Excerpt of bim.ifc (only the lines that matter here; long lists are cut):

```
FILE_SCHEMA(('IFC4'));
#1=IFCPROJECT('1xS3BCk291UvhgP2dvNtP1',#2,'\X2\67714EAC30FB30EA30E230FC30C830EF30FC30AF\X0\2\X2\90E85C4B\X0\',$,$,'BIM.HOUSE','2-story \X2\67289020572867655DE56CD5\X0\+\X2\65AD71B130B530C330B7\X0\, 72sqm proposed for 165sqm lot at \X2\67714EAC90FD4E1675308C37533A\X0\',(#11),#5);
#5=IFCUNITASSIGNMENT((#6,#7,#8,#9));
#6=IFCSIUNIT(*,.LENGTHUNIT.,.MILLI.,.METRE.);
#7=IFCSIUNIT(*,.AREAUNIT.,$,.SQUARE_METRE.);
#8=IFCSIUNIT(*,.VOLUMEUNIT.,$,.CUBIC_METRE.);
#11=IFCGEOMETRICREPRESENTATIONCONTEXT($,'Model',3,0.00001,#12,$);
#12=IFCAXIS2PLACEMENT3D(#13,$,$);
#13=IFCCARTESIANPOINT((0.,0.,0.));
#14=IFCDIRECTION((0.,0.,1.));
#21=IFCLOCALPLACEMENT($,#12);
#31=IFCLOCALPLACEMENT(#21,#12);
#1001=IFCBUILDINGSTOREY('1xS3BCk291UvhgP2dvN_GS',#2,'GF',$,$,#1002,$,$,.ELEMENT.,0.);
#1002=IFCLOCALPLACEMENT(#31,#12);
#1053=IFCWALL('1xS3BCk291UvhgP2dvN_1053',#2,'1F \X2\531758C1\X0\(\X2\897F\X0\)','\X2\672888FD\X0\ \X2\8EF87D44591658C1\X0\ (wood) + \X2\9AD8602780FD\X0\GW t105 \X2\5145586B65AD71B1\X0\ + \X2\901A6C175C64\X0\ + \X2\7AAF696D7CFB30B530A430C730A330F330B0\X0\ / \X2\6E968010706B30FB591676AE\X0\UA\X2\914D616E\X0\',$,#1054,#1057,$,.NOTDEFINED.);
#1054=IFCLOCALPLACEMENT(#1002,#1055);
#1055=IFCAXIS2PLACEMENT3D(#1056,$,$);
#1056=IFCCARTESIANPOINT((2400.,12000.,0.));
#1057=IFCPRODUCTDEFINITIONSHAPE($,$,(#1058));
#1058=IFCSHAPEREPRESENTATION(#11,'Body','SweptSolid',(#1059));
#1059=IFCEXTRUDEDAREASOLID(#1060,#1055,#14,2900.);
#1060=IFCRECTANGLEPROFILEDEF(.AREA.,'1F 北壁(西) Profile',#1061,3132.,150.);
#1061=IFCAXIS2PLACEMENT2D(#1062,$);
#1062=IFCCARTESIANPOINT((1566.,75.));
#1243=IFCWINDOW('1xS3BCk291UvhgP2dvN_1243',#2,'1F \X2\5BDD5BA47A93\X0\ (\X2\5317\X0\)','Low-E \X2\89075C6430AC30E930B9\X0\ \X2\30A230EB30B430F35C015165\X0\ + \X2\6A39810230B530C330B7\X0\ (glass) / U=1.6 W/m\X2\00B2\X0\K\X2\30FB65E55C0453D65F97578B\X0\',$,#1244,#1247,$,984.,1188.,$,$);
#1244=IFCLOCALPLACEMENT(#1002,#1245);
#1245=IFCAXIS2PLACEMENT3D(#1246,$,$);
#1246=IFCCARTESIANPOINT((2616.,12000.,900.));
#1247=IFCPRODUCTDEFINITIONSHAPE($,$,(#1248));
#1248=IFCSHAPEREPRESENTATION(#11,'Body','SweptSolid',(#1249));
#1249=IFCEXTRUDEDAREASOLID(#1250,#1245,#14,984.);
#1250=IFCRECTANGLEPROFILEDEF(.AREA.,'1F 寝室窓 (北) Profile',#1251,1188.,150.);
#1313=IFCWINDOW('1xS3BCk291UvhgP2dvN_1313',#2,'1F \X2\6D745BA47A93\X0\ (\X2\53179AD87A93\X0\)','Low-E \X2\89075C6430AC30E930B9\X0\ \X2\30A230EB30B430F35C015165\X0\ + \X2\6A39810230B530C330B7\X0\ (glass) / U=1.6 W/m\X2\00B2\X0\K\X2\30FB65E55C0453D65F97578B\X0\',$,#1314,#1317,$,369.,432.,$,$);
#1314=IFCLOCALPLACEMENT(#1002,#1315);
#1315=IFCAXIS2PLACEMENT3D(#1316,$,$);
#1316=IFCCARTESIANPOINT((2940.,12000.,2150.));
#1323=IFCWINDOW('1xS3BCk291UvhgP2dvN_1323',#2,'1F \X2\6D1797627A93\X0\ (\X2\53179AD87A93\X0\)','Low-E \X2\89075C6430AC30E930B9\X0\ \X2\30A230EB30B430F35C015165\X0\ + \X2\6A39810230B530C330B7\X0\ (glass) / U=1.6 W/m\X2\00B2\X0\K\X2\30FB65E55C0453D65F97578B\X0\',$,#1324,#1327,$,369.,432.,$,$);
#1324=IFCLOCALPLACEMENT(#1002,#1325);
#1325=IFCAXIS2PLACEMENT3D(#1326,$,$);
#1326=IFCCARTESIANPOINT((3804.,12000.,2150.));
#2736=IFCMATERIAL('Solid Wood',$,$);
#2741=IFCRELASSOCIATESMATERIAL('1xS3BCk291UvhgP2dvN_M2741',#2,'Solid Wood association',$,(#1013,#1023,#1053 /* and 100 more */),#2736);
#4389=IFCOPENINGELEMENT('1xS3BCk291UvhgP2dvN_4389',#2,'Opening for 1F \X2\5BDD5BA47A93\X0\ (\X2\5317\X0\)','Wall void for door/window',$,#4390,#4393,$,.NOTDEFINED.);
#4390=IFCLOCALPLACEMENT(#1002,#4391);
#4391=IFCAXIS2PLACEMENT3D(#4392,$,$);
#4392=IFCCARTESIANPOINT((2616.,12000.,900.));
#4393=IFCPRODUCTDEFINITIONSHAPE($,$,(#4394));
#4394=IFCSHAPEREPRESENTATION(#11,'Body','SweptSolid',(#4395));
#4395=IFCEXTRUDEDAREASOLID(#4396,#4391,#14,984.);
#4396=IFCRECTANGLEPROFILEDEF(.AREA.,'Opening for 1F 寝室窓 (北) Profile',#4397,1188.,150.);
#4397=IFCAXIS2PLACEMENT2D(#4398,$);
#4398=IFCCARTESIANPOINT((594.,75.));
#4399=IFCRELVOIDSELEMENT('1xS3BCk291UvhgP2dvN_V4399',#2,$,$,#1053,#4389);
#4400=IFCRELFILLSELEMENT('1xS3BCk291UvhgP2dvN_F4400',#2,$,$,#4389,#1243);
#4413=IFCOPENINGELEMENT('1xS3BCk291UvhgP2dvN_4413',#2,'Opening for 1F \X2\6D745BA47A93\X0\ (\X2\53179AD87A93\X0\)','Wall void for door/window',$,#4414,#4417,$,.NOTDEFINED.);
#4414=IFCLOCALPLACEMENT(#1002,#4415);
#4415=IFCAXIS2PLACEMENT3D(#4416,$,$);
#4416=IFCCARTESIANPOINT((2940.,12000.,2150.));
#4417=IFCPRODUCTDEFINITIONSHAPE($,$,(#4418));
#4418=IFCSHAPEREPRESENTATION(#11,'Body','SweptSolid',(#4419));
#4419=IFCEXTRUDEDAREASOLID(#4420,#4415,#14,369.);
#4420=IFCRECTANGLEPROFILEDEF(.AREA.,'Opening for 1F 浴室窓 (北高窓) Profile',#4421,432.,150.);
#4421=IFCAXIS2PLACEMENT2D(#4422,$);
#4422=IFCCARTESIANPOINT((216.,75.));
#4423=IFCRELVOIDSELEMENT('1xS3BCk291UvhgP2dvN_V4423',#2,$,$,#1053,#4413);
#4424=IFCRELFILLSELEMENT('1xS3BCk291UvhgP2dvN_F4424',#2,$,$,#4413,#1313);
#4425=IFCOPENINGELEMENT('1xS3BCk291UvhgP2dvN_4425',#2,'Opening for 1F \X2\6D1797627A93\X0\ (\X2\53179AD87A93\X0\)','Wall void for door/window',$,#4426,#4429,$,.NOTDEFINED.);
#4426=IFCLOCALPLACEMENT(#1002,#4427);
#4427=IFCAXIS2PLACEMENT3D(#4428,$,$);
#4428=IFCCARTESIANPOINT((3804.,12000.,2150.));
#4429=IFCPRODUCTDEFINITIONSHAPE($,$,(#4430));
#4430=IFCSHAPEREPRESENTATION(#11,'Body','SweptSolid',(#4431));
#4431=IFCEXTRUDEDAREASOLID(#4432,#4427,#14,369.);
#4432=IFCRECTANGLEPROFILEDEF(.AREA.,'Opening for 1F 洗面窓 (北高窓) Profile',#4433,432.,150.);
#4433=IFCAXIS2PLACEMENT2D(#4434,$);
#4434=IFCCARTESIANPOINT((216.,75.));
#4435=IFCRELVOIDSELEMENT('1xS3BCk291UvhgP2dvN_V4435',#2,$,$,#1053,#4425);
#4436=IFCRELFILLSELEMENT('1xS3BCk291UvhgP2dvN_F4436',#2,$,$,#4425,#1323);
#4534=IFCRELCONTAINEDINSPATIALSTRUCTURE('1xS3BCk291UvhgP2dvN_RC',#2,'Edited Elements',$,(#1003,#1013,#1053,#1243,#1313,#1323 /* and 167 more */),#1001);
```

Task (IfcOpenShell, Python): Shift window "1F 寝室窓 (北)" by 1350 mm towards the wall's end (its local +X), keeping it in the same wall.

```python
import ifcopenshell
import ifcopenshell.api.geometry
import ifcopenshell.util.placement
import ifcopenshell.util.unit

model = ifcopenshell.open("bim.ifc")
unit_scale = ifcopenshell.util.unit.calculate_unit_scale(model)

window = model.by_guid("1xS3BCk291UvhgP2dvN_1243")
opening = window.FillsVoids[0].RelatingOpeningElement
wall = opening.VoidsElements[0].RelatingBuildingElement

wall_matrix = ifcopenshell.util.placement.get_local_placement(wall.ObjectPlacement)
shift = wall_matrix[:3, 0] * 1.35 / unit_scale
before = ifcopenshell.util.placement.get_local_placement(window.ObjectPlacement)[:3, 3].copy()

# The window is not placed relative to its opening, so move both.
for product in (opening, window):
    matrix = ifcopenshell.util.placement.get_local_placement(product.ObjectPlacement)
    matrix[:3, 3] += shift
    ifcopenshell.api.geometry.edit_object_placement(model, product=product, matrix=matrix, is_si=False)

after = ifcopenshell.util.placement.get_local_placement(window.ObjectPlacement)[:3, 3]
print("window moved by", (after - before).round(3) + 0.0)

model.write("bim_v2.ifc")
```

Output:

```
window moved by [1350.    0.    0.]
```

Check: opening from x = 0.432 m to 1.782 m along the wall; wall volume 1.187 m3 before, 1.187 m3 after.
